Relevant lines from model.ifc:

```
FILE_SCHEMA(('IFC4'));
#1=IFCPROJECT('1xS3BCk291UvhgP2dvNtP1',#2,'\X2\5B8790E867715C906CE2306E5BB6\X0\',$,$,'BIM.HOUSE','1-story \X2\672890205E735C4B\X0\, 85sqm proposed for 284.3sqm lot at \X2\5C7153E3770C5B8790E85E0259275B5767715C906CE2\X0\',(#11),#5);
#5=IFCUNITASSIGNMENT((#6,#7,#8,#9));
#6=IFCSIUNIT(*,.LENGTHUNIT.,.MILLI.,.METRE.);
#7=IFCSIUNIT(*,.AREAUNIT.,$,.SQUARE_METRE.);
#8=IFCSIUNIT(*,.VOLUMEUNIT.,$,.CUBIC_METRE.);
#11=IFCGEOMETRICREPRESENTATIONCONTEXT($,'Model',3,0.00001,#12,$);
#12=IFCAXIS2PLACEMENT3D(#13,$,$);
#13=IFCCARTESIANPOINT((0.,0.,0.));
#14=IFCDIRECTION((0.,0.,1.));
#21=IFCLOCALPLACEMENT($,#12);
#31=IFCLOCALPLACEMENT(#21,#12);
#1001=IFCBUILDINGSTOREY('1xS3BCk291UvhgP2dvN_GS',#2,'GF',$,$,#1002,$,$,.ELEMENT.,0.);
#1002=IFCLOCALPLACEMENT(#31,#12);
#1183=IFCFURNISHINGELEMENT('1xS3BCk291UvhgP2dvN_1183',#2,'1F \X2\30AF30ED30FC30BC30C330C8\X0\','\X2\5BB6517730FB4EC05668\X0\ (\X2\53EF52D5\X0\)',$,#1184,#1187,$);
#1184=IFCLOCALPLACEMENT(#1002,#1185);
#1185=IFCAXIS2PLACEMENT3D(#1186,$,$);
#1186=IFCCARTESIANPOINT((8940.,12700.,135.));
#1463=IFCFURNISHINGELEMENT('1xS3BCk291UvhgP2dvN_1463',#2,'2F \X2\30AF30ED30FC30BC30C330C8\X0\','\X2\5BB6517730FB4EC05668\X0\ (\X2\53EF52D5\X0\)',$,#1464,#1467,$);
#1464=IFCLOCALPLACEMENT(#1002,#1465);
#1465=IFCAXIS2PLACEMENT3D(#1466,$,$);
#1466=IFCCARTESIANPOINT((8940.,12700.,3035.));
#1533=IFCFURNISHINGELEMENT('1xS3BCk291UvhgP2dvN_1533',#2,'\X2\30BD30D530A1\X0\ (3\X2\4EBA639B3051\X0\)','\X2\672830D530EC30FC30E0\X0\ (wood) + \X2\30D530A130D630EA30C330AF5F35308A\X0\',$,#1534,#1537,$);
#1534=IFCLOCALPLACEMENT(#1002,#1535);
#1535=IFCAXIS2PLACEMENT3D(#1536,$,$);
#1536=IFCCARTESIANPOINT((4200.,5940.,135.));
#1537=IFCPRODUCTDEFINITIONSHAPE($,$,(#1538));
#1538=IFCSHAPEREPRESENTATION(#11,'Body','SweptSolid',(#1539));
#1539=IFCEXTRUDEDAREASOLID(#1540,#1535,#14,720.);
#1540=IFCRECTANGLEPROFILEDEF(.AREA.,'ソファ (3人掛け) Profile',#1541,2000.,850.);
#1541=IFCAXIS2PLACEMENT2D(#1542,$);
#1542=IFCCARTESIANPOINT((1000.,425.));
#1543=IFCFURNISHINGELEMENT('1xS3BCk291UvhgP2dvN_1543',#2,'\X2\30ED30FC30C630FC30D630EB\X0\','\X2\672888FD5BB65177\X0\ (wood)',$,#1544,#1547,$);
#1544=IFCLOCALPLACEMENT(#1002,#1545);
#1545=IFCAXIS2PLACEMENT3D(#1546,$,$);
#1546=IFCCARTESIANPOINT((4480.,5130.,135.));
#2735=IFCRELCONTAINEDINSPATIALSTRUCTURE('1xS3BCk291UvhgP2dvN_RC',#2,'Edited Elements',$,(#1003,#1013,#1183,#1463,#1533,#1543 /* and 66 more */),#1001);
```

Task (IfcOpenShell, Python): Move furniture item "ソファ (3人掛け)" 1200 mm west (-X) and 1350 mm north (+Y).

```python
import ifcopenshell
import ifcopenshell.api.geometry
import ifcopenshell.util.placement
import ifcopenshell.util.unit

model = ifcopenshell.open("model.ifc")
unit_scale = ifcopenshell.util.unit.calculate_unit_scale(model)

item = model.by_id(1533)
matrix = ifcopenshell.util.placement.get_local_placement(item.ObjectPlacement)
matrix[0, 3] -= 1.2 / unit_scale
matrix[1, 3] += 1.35 / unit_scale
ifcopenshell.api.geometry.edit_object_placement(model, product=item, matrix=matrix, is_si=False)

print(ifcopenshell.util.placement.get_local_placement(item.ObjectPlacement).round(3) + 0.0)

model.write("model_edited.ifc")
```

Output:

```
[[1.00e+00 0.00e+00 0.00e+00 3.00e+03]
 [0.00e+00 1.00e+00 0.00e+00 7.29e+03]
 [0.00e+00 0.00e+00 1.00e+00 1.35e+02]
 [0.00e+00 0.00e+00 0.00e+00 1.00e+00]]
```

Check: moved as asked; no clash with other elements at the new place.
